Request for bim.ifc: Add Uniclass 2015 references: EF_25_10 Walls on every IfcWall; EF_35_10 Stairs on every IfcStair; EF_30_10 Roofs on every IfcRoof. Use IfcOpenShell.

First a look at what the model holds.

```python
import ifcopenshell

model = ifcopenshell.open("bim.ifc")
print(model.schema)
print("classifications:", [c.Name for c in model.by_type("IfcClassification")])
for ifc_class in ("IfcDoor", "IfcRoof", "IfcStair", "IfcWall", "IfcWindow"):
    print(ifc_class, len(model.by_type(ifc_class)))
```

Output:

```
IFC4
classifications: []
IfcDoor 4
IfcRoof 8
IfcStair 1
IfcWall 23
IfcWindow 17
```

```python
import ifcopenshell
import ifcopenshell.api.classification

model = ifcopenshell.open("bim.ifc")

system = ifcopenshell.api.classification.add_classification(model, classification="Uniclass 2015")

codes = {
    "IfcWall": ("EF_25_10", "Walls"),
    "IfcStair": ("EF_35_10", "Stairs"),
    "IfcRoof": ("EF_30_10", "Roofs"),
}
for ifc_class, (code, name) in codes.items():
    products = model.by_type(ifc_class)
    ifcopenshell.api.classification.add_reference(
        model, products=products, classification=system, identification=code, name=name
    )
    print(code, len(products))

model.write("bim_rev.ifc")
```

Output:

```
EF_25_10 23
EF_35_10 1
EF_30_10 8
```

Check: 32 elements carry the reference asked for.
